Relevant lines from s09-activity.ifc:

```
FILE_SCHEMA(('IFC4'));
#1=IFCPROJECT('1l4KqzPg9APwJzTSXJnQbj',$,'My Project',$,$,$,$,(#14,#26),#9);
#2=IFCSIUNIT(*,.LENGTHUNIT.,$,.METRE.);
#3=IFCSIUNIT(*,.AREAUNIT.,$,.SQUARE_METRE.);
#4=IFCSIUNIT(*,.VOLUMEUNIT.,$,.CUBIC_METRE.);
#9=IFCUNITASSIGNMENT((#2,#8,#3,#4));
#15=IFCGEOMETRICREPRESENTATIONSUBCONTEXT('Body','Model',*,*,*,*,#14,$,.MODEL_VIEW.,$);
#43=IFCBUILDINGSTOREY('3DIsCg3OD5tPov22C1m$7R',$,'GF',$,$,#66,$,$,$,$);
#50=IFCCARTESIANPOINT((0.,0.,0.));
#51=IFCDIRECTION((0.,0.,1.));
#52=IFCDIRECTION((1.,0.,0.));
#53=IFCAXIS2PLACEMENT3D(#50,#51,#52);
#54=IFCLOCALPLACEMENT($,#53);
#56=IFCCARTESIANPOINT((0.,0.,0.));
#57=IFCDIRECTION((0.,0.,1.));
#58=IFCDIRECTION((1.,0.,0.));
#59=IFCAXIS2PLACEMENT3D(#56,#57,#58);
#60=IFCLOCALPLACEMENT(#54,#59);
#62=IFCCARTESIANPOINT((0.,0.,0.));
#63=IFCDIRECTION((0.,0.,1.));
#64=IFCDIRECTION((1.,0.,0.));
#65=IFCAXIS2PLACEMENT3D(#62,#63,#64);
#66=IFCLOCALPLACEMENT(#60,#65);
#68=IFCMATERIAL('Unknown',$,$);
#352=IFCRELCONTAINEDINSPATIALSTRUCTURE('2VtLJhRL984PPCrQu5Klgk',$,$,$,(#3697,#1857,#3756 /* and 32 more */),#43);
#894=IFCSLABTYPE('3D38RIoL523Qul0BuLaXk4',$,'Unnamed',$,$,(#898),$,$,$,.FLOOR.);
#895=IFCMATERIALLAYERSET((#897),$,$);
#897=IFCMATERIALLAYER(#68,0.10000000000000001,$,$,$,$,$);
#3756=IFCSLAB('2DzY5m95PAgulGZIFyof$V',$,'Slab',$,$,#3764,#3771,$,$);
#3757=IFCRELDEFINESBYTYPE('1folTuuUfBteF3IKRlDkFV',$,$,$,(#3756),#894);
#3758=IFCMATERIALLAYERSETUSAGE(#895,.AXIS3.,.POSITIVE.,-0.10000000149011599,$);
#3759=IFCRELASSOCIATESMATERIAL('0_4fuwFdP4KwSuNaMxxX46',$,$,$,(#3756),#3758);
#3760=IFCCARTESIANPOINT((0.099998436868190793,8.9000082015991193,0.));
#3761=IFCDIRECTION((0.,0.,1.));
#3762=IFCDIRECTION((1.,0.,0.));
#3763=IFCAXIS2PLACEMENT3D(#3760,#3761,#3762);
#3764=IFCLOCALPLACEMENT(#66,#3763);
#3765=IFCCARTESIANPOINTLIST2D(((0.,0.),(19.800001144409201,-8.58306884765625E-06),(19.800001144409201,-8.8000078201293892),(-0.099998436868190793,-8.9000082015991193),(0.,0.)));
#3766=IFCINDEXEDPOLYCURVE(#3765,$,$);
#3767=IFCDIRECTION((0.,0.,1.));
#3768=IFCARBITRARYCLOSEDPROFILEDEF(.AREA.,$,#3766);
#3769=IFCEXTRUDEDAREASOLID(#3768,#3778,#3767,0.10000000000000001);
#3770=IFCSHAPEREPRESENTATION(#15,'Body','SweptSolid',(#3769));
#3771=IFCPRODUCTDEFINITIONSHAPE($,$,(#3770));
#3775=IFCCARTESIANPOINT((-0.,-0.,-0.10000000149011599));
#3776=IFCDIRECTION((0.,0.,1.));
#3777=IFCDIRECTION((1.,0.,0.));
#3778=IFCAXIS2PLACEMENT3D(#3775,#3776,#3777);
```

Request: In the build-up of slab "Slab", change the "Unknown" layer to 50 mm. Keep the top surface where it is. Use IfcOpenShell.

```python
import ifcopenshell
import ifcopenshell.util.element
import ifcopenshell.util.representation
import ifcopenshell.util.unit

model = ifcopenshell.open("s09-activity.ifc")
unit_scale = ifcopenshell.util.unit.calculate_unit_scale(model)

layer_set = model.by_id(895)
layer = next(l for l in layer_set.MaterialLayers if l.Material and l.Material.Name == "Unknown")
change = 0.05 / unit_scale - layer.LayerThickness
layer.LayerThickness += change

# Geometry does not follow the layer set by itself.
slabs = [e for e in ifcopenshell.util.element.get_elements_by_material(model, layer_set) if e.is_a("IfcSlab")]
for slab in sorted(slabs, key=lambda e: e.id()):
    body = ifcopenshell.util.representation.get_representation(slab, "Model", "Body")
    solid = body.Items[0]
    old_depth = solid.Depth
    solid.Depth += change
    # Extruded upwards: lower the start of the extrusion so the top stays.
    x, y, z = solid.Position.Location.Coordinates
    solid.Position.Location = model.createIfcCartesianPoint((x, y, z - change))
    print(slab.id(), f"{old_depth:g} -> {solid.Depth:g}")

# The layers are counted up from the underside, which has moved.
for usage in {ifcopenshell.util.element.get_material(slab) for slab in slabs}:
    usage.OffsetFromReferenceLine -= change

model.write("s09-activity_rev.ifc")
```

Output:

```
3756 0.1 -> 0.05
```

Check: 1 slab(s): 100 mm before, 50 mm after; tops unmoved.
